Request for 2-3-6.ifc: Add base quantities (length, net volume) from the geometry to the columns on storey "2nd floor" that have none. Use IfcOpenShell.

First a look at what the model holds.

```python
import ifcopenshell
import ifcopenshell.util.element
import ifcopenshell.util.unit

model = ifcopenshell.open("2-3-6.ifc")
print(model.schema)
for unit_type in ("LENGTHUNIT", "AREAUNIT", "VOLUMEUNIT"):
    print(unit_type, ifcopenshell.util.unit.calculate_unit_scale(model, unit_type))
storey = next(s for s in model.by_type("IfcBuildingStorey") if s.Name == "2nd floor")
columns = [e for e in ifcopenshell.util.element.get_decomposition(storey) if e.is_a("IfcColumn")]
for e in sorted(columns, key=lambda e: e.id()):
    print(e.id(), e.is_a(), e.Name, list(ifcopenshell.util.element.get_psets(e, qtos_only=True)), sep=" | ")
```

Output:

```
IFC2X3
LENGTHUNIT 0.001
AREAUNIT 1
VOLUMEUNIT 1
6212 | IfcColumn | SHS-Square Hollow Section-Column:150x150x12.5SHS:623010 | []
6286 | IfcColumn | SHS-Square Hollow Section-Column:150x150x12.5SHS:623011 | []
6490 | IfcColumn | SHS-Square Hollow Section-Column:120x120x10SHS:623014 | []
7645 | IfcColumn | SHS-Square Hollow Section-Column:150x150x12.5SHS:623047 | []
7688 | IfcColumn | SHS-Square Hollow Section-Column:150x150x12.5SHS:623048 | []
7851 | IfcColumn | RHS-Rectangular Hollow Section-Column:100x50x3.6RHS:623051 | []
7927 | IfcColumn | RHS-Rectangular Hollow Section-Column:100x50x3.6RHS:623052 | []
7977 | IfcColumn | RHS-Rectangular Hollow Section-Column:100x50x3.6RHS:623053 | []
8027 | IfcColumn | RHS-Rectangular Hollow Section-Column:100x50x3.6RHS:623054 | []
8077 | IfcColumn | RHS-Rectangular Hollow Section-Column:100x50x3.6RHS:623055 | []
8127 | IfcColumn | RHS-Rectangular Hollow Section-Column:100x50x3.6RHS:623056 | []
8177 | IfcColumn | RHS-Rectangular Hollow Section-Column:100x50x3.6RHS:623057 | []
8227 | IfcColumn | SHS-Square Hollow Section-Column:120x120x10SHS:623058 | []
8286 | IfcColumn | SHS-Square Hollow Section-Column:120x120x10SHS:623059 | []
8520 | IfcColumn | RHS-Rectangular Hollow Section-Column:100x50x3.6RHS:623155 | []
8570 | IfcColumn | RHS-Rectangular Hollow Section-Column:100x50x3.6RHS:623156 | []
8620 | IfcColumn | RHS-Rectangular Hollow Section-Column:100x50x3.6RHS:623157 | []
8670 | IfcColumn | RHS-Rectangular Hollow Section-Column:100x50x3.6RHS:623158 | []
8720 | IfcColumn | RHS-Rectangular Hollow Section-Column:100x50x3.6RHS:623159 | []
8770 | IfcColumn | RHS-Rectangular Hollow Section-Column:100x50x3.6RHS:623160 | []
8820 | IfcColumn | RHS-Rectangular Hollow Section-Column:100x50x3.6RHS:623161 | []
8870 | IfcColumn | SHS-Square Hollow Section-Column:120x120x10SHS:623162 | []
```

```python
import ifcopenshell
import ifcopenshell.api.pset
import ifcopenshell.geom
import ifcopenshell.util.element
import ifcopenshell.util.shape
import ifcopenshell.util.unit

model = ifcopenshell.open("2-3-6.ifc")
unit_scale = ifcopenshell.util.unit.calculate_unit_scale(model)
volume_scale = ifcopenshell.util.unit.calculate_unit_scale(model, "VOLUMEUNIT")
settings = ifcopenshell.geom.settings()

storey = next(s for s in model.by_type("IfcBuildingStorey") if s.Name == "2nd floor")
columns = [e for e in ifcopenshell.util.element.get_decomposition(storey) if e.is_a("IfcColumn")]

for e in sorted(columns, key=lambda e: e.id()):
    if ifcopenshell.util.element.get_psets(e, qtos_only=True, should_inherit=False):
        continue
    # Geometry comes back in metres, in the element's own axes.
    shape = ifcopenshell.geom.create_shape(settings, e)
    values = {
        "Length": ifcopenshell.util.shape.get_z(shape.geometry) / unit_scale,
        "NetVolume": ifcopenshell.util.shape.get_volume(shape.geometry) / volume_scale,
    }
    qto = ifcopenshell.api.pset.add_qto(model, product=e, name="BaseQuantities")
    ifcopenshell.api.pset.edit_qto(model, qto=qto, properties=values)
    print(e.id(), {k: round(v, 3) for k, v in values.items()})

model.write("2-3-6_rev.ifc")
```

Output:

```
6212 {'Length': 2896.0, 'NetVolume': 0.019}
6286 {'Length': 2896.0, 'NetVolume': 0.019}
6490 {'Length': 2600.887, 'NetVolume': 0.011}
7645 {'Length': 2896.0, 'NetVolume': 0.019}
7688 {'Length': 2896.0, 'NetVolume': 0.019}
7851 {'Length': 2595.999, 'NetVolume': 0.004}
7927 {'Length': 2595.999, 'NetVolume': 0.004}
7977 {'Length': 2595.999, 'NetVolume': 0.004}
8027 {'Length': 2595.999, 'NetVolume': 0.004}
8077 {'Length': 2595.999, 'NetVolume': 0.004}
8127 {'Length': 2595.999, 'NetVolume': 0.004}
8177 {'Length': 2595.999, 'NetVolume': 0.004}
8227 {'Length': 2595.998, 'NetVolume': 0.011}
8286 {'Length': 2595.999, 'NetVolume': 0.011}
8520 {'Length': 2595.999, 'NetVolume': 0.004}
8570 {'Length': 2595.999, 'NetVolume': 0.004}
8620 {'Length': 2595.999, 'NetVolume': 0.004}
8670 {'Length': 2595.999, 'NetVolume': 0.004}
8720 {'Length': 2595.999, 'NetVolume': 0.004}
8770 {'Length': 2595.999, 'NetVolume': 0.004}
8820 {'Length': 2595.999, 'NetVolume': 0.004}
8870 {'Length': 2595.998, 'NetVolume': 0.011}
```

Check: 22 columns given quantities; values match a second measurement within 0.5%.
